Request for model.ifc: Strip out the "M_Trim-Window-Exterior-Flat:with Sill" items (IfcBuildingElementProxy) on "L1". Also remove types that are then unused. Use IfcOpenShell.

First a look at what the model holds.

```python
import ifcopenshell
import ifcopenshell.util.element

model = ifcopenshell.open("model.ifc")
print(model.schema)
storey = next(s for s in model.by_type("IfcBuildingStorey") if s.Name == "L1")
proxies = [e for e in ifcopenshell.util.element.get_decomposition(storey) if e.is_a("IfcBuildingElementProxy")]
seen = {}
for e in proxies:
    element_type = ifcopenshell.util.element.get_type(e)
    name = element_type.Name if element_type not in (None, e) else None
    seen[name] = seen.get(name, 0) + 1
for name, count in sorted(seen.items(), key=str):
    print(count, "x", name)
```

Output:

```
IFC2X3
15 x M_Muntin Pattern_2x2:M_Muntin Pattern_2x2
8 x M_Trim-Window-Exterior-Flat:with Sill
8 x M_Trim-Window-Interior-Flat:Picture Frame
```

```python
import ifcopenshell
import ifcopenshell.api.root
import ifcopenshell.util.element

model = ifcopenshell.open("model.ifc")

storey = next(s for s in model.by_type("IfcBuildingStorey") if s.Name == "L1")
proxies = [e for e in ifcopenshell.util.element.get_decomposition(storey) if e.is_a("IfcBuildingElementProxy")]
targets = [e for e in proxies if (t := ifcopenshell.util.element.get_type(e)) not in (None, e) and t.Name == "M_Trim-Window-Exterior-Flat:with Sill"]
types = {ifcopenshell.util.element.get_type(e) for e in targets} - {None, *targets}

for e in targets:
    ifcopenshell.api.root.remove_product(model, product=e)
print(len(targets), "removed")

unused = [t for t in types if not ifcopenshell.util.element.get_types(t)]
for t in unused:
    ifcopenshell.api.root.remove_product(model, product=t)
print(len(unused), "unused types removed")

model.write("model_v2.ifc")
```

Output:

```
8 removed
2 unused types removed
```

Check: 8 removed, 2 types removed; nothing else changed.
